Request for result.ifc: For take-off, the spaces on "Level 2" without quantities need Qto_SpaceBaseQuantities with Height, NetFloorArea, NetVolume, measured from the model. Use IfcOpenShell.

First a look at what the model holds.

```python
import ifcopenshell
import ifcopenshell.util.element
import ifcopenshell.util.unit

model = ifcopenshell.open("result.ifc")
print(model.schema)
for unit_type in ("LENGTHUNIT", "AREAUNIT", "VOLUMEUNIT"):
    print(unit_type, ifcopenshell.util.unit.calculate_unit_scale(model, unit_type))
storey = next(s for s in model.by_type("IfcBuildingStorey") if s.Name == "Level 2")
spaces = [e for e in ifcopenshell.util.element.get_decomposition(storey) if e.is_a("IfcSpace")]
for e in sorted(spaces, key=lambda e: e.id()):
    print(e.id(), e.is_a(), e.Name, list(ifcopenshell.util.element.get_psets(e, qtos_only=True)), sep=" | ")
```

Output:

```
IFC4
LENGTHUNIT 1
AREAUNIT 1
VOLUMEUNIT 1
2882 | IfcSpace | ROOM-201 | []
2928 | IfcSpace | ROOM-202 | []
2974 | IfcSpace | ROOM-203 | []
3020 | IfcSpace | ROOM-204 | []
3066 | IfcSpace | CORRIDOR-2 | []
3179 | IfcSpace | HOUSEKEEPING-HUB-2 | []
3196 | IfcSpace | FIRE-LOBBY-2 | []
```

```python
import ifcopenshell
import ifcopenshell.api.pset
import ifcopenshell.geom
import ifcopenshell.util.element
import ifcopenshell.util.shape
import ifcopenshell.util.unit

model = ifcopenshell.open("result.ifc")
unit_scale = ifcopenshell.util.unit.calculate_unit_scale(model)
area_scale = ifcopenshell.util.unit.calculate_unit_scale(model, "AREAUNIT")
volume_scale = ifcopenshell.util.unit.calculate_unit_scale(model, "VOLUMEUNIT")
settings = ifcopenshell.geom.settings()

storey = next(s for s in model.by_type("IfcBuildingStorey") if s.Name == "Level 2")
spaces = [e for e in ifcopenshell.util.element.get_decomposition(storey) if e.is_a("IfcSpace")]

for e in sorted(spaces, key=lambda e: e.id()):
    if ifcopenshell.util.element.get_psets(e, qtos_only=True, should_inherit=False):
        continue
    # Geometry comes back in metres, in the element's own axes.
    shape = ifcopenshell.geom.create_shape(settings, e)
    values = {
        "Height": ifcopenshell.util.shape.get_z(shape.geometry) / unit_scale,
        "NetFloorArea": ifcopenshell.util.shape.get_footprint_area(shape.geometry) / area_scale,
        "NetVolume": ifcopenshell.util.shape.get_volume(shape.geometry) / volume_scale,
    }
    qto = ifcopenshell.api.pset.add_qto(model, product=e, name="Qto_SpaceBaseQuantities")
    ifcopenshell.api.pset.edit_qto(model, qto=qto, properties=values)
    print(e.id(), {k: round(v, 3) for k, v in values.items()})

model.write("result_updated.ifc")
```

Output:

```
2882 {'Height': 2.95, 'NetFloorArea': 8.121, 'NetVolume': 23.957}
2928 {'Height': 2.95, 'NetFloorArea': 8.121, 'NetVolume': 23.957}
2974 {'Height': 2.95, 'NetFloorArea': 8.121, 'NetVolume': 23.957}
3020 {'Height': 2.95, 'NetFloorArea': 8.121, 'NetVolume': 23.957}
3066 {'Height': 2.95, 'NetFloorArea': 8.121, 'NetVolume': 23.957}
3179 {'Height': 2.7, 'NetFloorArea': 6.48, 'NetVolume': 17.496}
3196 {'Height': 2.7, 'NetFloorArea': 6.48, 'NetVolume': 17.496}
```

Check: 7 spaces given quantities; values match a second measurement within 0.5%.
